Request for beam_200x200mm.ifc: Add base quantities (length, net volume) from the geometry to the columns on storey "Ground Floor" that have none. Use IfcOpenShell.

First a look at what the model holds.

```python
import ifcopenshell
import ifcopenshell.util.element
import ifcopenshell.util.unit

model = ifcopenshell.open("beam_200x200mm.ifc")
print(model.schema)
for unit_type in ("LENGTHUNIT", "AREAUNIT", "VOLUMEUNIT"):
    print(unit_type, ifcopenshell.util.unit.calculate_unit_scale(model, unit_type))
storey = next(s for s in model.by_type("IfcBuildingStorey") if s.Name == "Ground Floor")
columns = [e for e in ifcopenshell.util.element.get_decomposition(storey) if e.is_a("IfcColumn")]
for e in sorted(columns, key=lambda e: e.id()):
    print(e.id(), e.is_a(), e.Name, list(ifcopenshell.util.element.get_psets(e, qtos_only=True)), sep=" | ")
```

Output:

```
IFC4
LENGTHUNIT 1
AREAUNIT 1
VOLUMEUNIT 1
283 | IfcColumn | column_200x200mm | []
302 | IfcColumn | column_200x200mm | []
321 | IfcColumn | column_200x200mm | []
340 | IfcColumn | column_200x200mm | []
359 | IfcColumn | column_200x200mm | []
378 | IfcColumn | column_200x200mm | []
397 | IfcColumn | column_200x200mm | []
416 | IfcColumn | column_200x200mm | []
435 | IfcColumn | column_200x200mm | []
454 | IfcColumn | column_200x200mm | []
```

```python
import ifcopenshell
import ifcopenshell.api.pset
import ifcopenshell.geom
import ifcopenshell.util.element
import ifcopenshell.util.shape
import ifcopenshell.util.unit

model = ifcopenshell.open("beam_200x200mm.ifc")
unit_scale = ifcopenshell.util.unit.calculate_unit_scale(model)
volume_scale = ifcopenshell.util.unit.calculate_unit_scale(model, "VOLUMEUNIT")
settings = ifcopenshell.geom.settings()

storey = next(s for s in model.by_type("IfcBuildingStorey") if s.Name == "Ground Floor")
columns = [e for e in ifcopenshell.util.element.get_decomposition(storey) if e.is_a("IfcColumn")]

for e in sorted(columns, key=lambda e: e.id()):
    if ifcopenshell.util.element.get_psets(e, qtos_only=True, should_inherit=False):
        continue
    # Geometry comes back in metres, in the element's own axes.
    shape = ifcopenshell.geom.create_shape(settings, e)
    values = {
        "Length": ifcopenshell.util.shape.get_z(shape.geometry) / unit_scale,
        "NetVolume": ifcopenshell.util.shape.get_volume(shape.geometry) / volume_scale,
    }
    qto = ifcopenshell.api.pset.add_qto(model, product=e, name="Qto_ColumnBaseQuantities")
    ifcopenshell.api.pset.edit_qto(model, qto=qto, properties=values)
    print(e.id(), {k: round(v, 3) for k, v in values.items()})

model.write("beam_200x200mm_edited.ifc")
```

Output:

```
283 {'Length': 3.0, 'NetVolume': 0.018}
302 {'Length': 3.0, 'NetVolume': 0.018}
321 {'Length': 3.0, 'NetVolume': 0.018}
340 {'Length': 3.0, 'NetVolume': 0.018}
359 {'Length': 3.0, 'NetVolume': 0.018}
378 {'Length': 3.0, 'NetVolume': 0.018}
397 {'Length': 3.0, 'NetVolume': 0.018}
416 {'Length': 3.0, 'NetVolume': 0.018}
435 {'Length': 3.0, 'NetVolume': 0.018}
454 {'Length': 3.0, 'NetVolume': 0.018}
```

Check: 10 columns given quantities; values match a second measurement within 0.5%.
